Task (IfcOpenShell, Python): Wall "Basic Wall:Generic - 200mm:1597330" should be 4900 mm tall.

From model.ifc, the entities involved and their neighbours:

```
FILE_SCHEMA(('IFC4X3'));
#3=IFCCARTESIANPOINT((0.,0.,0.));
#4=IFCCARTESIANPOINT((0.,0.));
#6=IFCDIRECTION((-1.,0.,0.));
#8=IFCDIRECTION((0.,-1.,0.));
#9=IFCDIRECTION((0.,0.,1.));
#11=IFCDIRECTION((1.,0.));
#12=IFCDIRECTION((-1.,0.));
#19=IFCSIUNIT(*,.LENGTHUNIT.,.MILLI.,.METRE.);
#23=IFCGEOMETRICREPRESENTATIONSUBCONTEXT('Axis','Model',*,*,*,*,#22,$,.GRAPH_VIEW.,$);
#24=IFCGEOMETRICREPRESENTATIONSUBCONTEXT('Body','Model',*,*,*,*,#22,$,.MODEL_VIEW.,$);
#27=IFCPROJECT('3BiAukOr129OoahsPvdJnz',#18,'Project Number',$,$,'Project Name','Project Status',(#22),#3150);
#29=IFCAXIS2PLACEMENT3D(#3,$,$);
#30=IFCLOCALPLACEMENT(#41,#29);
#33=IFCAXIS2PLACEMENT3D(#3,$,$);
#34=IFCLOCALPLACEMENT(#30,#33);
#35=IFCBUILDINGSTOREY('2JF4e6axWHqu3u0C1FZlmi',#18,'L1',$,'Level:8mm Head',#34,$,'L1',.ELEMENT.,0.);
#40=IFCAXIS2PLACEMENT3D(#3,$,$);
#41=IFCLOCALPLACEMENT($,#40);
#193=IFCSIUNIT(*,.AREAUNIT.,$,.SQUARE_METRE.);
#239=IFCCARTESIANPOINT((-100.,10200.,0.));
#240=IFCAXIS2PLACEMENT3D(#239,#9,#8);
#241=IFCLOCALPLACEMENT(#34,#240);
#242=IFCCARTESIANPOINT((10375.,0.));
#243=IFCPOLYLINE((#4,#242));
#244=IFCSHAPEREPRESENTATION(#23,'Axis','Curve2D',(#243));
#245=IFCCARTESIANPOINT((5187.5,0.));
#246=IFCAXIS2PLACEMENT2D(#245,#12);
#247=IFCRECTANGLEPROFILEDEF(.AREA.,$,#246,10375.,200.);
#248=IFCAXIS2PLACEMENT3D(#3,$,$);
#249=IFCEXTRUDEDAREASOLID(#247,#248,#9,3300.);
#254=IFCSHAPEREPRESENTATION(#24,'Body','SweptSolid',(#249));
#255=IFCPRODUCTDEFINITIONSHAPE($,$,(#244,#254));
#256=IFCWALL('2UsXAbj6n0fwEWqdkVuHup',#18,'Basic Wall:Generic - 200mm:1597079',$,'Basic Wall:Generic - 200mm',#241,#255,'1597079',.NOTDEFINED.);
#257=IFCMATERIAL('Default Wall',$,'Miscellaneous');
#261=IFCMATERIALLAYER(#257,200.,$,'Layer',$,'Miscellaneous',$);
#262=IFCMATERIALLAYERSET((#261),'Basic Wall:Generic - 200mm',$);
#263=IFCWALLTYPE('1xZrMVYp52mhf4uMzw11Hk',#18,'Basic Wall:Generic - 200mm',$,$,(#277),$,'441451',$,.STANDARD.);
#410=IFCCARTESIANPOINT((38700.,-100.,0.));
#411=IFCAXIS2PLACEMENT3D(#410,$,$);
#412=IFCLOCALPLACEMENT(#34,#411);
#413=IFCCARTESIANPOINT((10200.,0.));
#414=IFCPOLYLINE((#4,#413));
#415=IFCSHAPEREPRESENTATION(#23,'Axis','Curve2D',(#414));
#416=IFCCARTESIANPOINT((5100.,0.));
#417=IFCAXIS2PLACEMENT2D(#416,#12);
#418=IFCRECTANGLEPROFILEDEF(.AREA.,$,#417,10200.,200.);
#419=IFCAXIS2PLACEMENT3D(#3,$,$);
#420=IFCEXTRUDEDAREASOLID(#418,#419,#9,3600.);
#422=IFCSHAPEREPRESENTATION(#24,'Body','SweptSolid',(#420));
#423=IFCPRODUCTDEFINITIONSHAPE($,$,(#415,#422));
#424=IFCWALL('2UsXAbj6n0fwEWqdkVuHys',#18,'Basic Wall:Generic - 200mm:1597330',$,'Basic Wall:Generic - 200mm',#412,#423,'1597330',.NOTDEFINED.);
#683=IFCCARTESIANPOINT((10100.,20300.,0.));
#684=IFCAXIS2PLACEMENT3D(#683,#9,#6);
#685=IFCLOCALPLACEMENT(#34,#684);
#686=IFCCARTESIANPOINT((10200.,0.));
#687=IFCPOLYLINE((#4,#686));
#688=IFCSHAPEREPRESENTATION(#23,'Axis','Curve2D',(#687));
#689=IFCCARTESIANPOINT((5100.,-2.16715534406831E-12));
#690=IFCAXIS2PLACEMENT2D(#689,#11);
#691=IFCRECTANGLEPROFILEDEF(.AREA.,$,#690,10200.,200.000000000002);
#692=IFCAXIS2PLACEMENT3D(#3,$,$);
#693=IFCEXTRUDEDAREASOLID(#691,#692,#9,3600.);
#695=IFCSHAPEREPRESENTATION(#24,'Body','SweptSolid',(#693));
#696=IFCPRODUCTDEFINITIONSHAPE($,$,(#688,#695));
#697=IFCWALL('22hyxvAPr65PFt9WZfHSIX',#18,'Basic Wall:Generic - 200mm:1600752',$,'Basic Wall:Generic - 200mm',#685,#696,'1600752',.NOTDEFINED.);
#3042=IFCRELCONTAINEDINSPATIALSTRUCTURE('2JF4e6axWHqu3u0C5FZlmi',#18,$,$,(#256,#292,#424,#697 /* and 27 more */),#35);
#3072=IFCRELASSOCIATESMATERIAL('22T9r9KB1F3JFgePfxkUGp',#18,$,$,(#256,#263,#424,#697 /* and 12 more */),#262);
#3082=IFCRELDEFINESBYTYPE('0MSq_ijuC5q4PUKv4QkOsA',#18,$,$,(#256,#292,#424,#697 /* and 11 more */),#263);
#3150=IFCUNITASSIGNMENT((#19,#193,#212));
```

```python
import ifcopenshell
import ifcopenshell.geom
import ifcopenshell.util.representation
import ifcopenshell.util.shape
import ifcopenshell.util.unit

model = ifcopenshell.open("model.ifc")
unit_scale = ifcopenshell.util.unit.calculate_unit_scale(model)
settings = ifcopenshell.geom.settings()


def volume(element):
    """Net volume in cubic metres, openings subtracted."""
    shape = ifcopenshell.geom.create_shape(settings, element)
    return ifcopenshell.util.shape.get_volume(shape.geometry)


wall = model.by_id(424)
before = volume(wall)

body = ifcopenshell.util.representation.get_representation(wall, "Model", "Body")
solid = body.Items[0]
old_height = solid.Depth
solid.Depth = 4.9 / unit_scale
after = volume(wall)

print(f"height {old_height:g} -> {solid.Depth:g}, volume {before:.3f} -> {after:.3f} m3")

model.write("model_edited.ifc")
```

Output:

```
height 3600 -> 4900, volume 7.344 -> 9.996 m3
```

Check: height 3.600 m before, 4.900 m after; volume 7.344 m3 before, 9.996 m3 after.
